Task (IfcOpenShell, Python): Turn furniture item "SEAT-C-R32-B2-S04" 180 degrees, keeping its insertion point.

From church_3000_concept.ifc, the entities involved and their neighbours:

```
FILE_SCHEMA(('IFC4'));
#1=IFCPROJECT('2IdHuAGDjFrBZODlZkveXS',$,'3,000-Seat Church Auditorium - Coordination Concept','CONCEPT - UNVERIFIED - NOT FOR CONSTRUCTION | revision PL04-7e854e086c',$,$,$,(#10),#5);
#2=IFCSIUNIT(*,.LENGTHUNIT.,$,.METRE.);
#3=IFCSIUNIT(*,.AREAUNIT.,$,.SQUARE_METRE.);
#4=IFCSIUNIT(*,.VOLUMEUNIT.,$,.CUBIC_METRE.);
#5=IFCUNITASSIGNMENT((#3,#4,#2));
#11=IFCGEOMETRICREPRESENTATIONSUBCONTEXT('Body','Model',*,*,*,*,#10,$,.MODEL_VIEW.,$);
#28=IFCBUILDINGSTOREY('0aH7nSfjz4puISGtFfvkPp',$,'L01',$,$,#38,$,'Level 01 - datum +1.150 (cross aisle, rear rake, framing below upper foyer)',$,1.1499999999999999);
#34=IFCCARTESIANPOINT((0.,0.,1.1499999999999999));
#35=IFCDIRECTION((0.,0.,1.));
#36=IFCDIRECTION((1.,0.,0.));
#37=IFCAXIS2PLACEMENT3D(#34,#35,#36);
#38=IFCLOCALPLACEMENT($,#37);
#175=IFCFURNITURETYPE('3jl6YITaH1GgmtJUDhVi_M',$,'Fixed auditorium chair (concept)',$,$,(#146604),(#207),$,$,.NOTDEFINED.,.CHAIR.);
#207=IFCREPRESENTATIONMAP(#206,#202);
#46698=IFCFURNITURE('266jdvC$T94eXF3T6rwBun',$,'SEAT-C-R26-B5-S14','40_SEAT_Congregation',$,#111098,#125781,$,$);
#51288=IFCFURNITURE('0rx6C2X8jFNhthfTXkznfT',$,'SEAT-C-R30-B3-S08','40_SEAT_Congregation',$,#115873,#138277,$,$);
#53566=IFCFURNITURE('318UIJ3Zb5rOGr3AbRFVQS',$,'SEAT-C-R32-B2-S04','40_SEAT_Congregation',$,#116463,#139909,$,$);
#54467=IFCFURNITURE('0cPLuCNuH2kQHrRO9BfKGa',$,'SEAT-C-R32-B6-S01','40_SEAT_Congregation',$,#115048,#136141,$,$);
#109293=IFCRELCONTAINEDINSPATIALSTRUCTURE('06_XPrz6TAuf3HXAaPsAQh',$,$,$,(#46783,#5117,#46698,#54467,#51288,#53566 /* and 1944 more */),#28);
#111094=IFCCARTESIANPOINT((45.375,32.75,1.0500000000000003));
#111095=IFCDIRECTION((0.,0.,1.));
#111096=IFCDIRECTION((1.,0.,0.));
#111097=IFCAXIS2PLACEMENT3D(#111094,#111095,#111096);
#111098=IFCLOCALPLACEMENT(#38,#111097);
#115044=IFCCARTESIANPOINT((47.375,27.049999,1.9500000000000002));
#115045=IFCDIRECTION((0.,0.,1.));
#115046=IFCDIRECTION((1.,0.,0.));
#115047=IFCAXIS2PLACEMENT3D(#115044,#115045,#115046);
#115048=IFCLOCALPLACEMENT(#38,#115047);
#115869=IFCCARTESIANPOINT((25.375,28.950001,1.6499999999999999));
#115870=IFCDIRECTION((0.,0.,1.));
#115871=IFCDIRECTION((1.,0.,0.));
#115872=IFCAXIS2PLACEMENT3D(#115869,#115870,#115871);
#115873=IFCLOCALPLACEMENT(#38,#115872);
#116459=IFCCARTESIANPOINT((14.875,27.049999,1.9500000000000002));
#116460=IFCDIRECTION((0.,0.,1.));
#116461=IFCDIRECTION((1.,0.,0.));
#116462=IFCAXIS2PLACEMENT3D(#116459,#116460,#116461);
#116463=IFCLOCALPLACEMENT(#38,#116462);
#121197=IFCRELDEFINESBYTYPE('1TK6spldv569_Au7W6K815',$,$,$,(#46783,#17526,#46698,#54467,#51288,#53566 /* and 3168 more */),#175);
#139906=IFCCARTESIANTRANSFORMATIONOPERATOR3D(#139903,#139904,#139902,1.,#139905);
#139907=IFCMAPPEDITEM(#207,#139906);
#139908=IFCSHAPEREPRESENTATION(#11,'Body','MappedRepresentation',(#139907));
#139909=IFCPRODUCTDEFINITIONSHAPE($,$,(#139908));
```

```python
import ifcopenshell
import ifcopenshell.api.geometry
import ifcopenshell.util.placement

model = ifcopenshell.open("church_3000_concept.ifc")

item = model.by_guid("318UIJ3Zb5rOGr3AbRFVQS")
matrix = ifcopenshell.util.placement.get_local_placement(item.ObjectPlacement)
matrix = matrix @ ifcopenshell.util.placement.rotation(180, "Z")
ifcopenshell.api.geometry.edit_object_placement(model, product=item, matrix=matrix, is_si=False)

print(ifcopenshell.util.placement.get_local_placement(item.ObjectPlacement).round(3) + 0.0)

model.write("church_3000_concept_edited.ifc")
```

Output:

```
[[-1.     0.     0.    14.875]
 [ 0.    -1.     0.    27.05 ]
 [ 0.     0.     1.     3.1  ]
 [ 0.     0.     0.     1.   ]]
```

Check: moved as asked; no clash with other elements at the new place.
